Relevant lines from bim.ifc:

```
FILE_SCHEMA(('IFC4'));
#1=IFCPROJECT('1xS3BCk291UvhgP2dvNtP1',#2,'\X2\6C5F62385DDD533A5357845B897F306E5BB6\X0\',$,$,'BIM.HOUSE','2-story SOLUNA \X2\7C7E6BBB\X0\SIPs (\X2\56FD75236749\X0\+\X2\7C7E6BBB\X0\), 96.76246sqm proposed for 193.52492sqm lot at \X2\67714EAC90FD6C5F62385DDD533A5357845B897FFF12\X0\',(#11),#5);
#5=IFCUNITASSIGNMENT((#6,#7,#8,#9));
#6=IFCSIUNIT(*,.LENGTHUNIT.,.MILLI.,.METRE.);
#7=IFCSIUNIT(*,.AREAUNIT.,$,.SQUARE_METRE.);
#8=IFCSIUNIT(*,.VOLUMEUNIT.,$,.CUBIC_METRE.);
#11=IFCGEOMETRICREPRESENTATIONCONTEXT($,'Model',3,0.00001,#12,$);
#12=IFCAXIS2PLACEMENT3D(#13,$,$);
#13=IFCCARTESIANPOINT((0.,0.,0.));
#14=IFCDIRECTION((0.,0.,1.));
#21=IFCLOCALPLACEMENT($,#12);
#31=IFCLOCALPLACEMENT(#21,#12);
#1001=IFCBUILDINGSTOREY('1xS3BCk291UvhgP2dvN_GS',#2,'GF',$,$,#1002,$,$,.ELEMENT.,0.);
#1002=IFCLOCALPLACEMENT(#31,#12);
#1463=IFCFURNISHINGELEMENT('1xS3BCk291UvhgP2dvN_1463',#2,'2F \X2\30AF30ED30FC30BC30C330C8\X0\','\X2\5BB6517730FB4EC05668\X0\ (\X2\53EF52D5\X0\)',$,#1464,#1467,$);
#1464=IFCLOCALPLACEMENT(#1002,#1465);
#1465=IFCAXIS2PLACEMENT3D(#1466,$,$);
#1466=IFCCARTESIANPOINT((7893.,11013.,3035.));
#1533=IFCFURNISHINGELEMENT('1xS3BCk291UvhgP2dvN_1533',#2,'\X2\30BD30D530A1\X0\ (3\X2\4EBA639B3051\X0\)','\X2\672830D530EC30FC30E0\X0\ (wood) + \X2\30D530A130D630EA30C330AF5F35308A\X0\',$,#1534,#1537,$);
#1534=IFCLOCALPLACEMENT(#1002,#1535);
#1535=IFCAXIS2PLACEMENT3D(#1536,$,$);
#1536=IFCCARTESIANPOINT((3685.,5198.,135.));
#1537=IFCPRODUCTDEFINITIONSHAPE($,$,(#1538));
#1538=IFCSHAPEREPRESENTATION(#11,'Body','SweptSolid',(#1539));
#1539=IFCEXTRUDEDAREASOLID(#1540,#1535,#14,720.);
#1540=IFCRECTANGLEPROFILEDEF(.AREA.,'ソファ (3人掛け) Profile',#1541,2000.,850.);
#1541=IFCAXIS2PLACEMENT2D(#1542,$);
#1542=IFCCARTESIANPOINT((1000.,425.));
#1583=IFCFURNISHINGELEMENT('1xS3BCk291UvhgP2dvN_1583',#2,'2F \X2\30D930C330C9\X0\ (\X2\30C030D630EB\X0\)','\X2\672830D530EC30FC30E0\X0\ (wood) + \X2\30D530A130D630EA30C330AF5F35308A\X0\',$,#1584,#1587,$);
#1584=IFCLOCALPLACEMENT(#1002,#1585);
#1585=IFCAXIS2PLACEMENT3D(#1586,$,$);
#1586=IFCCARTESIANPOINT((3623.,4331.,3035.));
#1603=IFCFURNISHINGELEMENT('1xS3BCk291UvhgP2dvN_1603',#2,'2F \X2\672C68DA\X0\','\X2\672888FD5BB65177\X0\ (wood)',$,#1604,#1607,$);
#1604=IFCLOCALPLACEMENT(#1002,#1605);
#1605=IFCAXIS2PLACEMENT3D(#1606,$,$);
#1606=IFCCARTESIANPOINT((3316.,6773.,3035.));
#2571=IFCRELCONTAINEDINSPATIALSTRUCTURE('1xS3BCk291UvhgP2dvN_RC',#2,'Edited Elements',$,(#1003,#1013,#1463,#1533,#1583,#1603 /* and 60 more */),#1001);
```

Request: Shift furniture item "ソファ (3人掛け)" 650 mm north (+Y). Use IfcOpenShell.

```python
import ifcopenshell
import ifcopenshell.api.geometry
import ifcopenshell.util.placement
import ifcopenshell.util.unit

model = ifcopenshell.open("bim.ifc")
unit_scale = ifcopenshell.util.unit.calculate_unit_scale(model)

item = model.by_id(1533)
matrix = ifcopenshell.util.placement.get_local_placement(item.ObjectPlacement)
matrix[1, 3] += 0.65 / unit_scale
ifcopenshell.api.geometry.edit_object_placement(model, product=item, matrix=matrix, is_si=False)

print(ifcopenshell.util.placement.get_local_placement(item.ObjectPlacement).round(3) + 0.0)

model.write("bim_updated.ifc")
```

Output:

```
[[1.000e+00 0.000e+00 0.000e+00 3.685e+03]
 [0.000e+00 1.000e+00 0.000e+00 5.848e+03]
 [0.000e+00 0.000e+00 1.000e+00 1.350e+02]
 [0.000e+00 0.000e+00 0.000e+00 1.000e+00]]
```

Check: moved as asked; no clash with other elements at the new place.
